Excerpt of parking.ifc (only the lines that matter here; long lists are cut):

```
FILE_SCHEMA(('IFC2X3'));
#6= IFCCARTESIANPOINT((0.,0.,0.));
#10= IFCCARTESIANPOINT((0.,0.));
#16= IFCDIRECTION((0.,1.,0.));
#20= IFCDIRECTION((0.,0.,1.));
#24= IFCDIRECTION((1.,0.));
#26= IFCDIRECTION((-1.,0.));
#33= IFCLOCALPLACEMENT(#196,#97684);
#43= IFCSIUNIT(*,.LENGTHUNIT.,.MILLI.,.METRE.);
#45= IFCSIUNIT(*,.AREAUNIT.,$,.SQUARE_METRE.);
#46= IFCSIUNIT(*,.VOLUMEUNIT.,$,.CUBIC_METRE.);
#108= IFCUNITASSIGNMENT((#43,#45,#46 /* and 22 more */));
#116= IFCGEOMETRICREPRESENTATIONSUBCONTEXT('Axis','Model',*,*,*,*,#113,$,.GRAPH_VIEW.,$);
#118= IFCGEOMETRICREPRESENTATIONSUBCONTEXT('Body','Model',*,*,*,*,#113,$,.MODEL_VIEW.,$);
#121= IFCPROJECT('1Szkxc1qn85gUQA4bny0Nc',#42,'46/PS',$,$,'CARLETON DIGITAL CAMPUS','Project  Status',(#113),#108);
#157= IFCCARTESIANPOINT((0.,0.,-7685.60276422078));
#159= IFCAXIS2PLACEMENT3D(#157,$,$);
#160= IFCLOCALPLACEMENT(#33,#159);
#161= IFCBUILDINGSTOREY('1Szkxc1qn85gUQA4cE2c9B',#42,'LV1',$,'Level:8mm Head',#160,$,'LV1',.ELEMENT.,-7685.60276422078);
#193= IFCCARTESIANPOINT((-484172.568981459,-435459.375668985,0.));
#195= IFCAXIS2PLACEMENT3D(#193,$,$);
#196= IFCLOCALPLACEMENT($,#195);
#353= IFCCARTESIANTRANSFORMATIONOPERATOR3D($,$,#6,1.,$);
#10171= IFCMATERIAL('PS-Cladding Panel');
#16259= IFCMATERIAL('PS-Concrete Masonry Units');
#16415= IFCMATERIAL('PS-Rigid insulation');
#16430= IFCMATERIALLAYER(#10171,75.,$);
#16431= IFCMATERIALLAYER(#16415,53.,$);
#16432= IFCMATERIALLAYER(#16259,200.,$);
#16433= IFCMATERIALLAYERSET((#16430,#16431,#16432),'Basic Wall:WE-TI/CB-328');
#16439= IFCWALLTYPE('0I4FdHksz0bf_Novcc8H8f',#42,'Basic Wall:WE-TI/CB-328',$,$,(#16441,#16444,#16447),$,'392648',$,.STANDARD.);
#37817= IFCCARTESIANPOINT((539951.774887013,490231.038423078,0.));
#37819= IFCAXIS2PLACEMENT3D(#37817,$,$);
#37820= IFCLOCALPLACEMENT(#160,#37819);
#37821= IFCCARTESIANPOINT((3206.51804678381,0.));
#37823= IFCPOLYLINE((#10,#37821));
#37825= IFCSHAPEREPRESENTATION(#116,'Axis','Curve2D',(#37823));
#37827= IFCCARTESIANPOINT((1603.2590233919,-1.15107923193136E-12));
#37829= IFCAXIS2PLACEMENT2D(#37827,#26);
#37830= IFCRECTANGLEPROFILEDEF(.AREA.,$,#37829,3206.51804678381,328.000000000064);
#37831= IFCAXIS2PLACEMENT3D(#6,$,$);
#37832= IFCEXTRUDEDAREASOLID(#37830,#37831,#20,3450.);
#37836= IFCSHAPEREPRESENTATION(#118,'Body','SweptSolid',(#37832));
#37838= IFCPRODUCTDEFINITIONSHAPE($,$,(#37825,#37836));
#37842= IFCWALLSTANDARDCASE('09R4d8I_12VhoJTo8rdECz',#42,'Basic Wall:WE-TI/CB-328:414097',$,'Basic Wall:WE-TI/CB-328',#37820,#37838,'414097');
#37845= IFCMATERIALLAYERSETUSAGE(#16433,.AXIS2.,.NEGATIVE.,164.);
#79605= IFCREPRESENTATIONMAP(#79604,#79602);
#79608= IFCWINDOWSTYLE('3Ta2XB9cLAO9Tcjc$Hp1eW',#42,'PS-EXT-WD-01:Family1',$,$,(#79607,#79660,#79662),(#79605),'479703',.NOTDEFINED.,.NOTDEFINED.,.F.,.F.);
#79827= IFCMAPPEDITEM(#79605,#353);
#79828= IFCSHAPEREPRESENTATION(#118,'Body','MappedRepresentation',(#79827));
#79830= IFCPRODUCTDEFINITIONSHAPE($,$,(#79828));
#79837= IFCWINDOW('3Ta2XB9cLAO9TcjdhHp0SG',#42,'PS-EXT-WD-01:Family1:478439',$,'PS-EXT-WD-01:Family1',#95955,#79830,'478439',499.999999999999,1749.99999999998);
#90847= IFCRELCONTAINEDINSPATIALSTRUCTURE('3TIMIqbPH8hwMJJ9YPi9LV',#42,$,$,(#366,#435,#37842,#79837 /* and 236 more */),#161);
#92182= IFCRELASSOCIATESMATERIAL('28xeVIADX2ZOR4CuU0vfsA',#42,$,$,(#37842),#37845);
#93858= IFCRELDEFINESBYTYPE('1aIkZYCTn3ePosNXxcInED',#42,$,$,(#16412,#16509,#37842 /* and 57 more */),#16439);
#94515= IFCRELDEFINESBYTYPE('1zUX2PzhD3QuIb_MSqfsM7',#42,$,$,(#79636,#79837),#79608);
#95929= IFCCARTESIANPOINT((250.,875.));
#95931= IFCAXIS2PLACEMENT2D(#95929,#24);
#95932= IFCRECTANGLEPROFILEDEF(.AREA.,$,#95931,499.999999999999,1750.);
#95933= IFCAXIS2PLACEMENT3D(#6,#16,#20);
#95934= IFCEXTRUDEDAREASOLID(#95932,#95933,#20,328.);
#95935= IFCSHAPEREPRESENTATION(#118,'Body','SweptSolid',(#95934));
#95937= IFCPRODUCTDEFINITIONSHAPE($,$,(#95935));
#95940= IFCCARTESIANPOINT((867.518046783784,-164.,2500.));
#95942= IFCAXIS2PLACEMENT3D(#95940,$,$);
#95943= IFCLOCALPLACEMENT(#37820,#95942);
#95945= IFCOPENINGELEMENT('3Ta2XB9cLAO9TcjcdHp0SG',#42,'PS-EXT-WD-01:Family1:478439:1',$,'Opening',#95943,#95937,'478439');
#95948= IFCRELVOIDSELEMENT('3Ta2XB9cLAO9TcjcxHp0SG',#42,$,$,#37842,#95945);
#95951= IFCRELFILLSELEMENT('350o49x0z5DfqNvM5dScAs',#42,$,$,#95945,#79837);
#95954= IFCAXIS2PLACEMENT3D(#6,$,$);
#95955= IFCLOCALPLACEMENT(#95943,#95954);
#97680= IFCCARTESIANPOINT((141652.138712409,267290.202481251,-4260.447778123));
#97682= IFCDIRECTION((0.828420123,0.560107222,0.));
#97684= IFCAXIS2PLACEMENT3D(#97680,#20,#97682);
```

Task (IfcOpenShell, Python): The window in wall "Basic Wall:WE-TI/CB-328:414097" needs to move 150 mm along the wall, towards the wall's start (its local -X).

```python
import ifcopenshell
import ifcopenshell.api.geometry
import ifcopenshell.util.placement
import ifcopenshell.util.unit

model = ifcopenshell.open("parking.ifc")
unit_scale = ifcopenshell.util.unit.calculate_unit_scale(model)

window = model.by_guid("3Ta2XB9cLAO9TcjdhHp0SG")
opening = window.FillsVoids[0].RelatingOpeningElement
wall = opening.VoidsElements[0].RelatingBuildingElement

wall_matrix = ifcopenshell.util.placement.get_local_placement(wall.ObjectPlacement)
shift = wall_matrix[:3, 0] * -0.15 / unit_scale
before = ifcopenshell.util.placement.get_local_placement(window.ObjectPlacement)[:3, 3].copy()

# The window is placed relative to its opening, so it follows when the opening moves.
matrix = ifcopenshell.util.placement.get_local_placement(opening.ObjectPlacement)
matrix[:3, 3] += shift
ifcopenshell.api.geometry.edit_object_placement(
    model, product=opening, matrix=matrix, is_si=False, should_transform_children=True
)

after = ifcopenshell.util.placement.get_local_placement(window.ObjectPlacement)[:3, 3]
print("window moved by", (after - before).round(3) + 0.0)

model.write("parking_updated.ifc")
```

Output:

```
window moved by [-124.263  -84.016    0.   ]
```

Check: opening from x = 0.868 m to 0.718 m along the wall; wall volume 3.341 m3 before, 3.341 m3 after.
